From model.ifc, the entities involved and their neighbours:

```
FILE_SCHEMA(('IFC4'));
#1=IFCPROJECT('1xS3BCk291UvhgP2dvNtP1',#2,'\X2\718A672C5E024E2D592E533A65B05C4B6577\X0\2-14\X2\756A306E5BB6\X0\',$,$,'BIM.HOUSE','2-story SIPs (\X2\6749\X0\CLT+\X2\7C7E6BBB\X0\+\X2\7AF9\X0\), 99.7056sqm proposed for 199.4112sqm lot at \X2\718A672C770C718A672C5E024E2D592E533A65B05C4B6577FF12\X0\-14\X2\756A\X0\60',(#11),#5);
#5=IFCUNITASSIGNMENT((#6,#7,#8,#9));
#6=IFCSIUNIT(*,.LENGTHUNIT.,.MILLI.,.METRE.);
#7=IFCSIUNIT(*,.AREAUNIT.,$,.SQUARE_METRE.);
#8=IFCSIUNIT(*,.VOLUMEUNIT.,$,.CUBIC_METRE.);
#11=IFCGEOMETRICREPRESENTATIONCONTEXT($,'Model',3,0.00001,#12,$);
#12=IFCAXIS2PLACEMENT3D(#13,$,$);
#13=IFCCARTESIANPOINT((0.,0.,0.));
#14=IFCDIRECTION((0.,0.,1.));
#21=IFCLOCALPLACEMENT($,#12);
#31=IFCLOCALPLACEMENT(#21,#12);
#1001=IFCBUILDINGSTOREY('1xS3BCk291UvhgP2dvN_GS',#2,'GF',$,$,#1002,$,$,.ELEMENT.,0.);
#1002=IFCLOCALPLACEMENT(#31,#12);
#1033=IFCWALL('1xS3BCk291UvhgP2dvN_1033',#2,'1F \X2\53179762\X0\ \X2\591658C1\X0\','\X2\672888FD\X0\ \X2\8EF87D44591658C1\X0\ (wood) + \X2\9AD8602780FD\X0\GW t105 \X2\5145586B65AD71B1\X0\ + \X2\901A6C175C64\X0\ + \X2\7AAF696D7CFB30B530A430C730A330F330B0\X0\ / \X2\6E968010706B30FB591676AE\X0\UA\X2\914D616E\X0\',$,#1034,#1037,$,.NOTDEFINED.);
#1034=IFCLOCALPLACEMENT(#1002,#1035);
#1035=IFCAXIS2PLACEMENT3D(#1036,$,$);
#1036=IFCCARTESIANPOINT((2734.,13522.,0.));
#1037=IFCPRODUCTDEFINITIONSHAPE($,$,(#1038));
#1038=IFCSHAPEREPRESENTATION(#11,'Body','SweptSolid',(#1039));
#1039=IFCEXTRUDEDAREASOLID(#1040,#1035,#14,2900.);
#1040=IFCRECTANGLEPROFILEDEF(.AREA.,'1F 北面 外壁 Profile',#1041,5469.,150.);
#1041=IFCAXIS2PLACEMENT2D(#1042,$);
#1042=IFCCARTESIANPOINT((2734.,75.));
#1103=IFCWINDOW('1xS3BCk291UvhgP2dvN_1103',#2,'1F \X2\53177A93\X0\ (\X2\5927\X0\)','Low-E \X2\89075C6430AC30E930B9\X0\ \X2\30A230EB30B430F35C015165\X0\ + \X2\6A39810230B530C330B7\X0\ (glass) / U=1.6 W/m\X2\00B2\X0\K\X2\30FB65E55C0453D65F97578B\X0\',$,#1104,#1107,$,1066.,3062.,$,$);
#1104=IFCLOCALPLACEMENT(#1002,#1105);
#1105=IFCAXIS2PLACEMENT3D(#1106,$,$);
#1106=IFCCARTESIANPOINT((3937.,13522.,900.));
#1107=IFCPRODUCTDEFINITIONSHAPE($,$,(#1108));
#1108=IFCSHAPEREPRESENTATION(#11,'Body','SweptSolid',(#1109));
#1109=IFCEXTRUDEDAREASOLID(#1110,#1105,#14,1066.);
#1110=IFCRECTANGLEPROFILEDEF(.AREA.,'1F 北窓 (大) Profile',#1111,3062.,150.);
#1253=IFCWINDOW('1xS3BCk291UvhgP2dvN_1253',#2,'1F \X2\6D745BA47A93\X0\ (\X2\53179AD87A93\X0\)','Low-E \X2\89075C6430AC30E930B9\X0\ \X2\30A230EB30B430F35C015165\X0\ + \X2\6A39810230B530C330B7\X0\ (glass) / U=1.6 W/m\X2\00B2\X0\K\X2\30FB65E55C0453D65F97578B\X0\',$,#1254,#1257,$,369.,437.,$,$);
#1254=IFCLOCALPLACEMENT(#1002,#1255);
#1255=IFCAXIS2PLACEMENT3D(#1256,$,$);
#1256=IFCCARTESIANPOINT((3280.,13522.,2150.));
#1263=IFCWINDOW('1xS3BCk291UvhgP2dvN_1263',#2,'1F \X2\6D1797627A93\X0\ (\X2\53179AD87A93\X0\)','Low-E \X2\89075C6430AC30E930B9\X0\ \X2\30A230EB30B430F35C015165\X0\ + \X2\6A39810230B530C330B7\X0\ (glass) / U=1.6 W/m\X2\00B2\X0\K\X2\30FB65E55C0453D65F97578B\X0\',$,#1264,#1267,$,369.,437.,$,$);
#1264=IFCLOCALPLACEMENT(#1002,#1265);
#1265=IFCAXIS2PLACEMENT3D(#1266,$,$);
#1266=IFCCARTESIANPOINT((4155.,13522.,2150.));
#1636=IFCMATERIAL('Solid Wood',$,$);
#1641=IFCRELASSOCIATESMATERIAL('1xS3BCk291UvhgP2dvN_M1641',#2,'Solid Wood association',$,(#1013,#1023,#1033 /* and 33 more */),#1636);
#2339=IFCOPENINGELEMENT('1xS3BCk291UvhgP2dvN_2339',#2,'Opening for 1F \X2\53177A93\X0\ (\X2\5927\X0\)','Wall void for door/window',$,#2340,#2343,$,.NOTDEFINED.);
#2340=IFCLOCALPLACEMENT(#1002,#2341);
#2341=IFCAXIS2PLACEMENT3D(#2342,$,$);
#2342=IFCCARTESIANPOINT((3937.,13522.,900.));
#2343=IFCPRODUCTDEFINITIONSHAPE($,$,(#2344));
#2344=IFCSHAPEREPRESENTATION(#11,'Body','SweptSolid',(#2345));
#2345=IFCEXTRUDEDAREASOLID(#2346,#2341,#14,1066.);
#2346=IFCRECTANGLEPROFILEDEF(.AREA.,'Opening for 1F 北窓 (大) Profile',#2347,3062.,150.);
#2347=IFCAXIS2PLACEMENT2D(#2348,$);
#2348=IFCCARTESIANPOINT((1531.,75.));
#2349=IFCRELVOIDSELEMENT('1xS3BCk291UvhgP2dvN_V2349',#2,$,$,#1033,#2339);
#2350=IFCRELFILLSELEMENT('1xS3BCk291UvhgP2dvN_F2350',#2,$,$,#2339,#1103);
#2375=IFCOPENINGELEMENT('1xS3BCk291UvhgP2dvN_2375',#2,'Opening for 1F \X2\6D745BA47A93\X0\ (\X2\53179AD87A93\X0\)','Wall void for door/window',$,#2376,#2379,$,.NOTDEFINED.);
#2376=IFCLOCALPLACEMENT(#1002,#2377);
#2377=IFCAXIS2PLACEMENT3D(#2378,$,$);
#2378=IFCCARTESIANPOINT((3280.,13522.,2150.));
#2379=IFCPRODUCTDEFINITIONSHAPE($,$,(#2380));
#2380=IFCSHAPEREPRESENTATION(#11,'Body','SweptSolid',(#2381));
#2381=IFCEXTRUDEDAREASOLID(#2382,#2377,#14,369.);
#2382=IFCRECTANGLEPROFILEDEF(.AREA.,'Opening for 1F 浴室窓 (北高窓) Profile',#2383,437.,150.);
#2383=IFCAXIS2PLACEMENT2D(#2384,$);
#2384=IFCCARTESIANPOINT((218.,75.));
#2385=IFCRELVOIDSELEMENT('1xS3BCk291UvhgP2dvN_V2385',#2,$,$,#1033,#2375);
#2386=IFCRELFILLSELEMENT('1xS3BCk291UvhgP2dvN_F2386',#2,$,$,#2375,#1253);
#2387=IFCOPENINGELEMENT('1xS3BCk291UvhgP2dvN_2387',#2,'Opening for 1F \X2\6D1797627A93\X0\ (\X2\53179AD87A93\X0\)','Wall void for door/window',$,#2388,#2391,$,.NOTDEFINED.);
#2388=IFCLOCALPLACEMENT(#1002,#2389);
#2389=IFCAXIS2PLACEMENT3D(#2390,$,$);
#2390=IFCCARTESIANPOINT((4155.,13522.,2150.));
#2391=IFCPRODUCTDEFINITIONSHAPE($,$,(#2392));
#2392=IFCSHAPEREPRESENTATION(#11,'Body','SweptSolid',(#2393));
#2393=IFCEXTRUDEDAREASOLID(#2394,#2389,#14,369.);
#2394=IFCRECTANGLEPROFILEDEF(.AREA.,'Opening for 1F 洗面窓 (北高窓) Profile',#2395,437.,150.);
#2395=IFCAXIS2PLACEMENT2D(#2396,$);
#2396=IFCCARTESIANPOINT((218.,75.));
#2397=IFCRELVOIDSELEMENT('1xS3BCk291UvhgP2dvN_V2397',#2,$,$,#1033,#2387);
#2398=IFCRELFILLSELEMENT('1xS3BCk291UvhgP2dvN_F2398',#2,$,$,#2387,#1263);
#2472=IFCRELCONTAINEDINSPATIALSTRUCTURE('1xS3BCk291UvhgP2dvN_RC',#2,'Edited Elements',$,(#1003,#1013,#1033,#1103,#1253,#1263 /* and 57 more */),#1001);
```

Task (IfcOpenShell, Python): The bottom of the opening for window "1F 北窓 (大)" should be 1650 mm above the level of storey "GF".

```python
import numpy as np
import ifcopenshell
import ifcopenshell.api.geometry
import ifcopenshell.geom
import ifcopenshell.util.element
import ifcopenshell.util.placement
import ifcopenshell.util.shape
import ifcopenshell.util.unit

model = ifcopenshell.open("model.ifc")
unit_scale = ifcopenshell.util.unit.calculate_unit_scale(model)

window = model.by_id(1103)
opening = window.FillsVoids[0].RelatingOpeningElement
storey = ifcopenshell.util.element.get_container(window, ifc_class="IfcBuildingStorey")
level = ifcopenshell.util.placement.get_local_placement(storey.ObjectPlacement)[2, 3]

# The opening's origin need not be at the sill, so measure its lowest point.
shape = ifcopenshell.geom.create_shape(ifcopenshell.geom.settings(), opening)
bottom = ifcopenshell.util.shape.get_shape_bottom_elevation(shape, shape.geometry) / unit_scale
dz = level + 1.65 / unit_scale - bottom

shift = np.array([0.0, 0.0, dz])
# The window is not placed relative to its opening, so move both.
for product in (opening, window):
    matrix = ifcopenshell.util.placement.get_local_placement(product.ObjectPlacement)
    matrix[:3, 3] += shift
    ifcopenshell.api.geometry.edit_object_placement(model, product=product, matrix=matrix, is_si=False)

print(f"moved by {dz * unit_scale:+.3f} m")

model.write("model_updated.ifc")
```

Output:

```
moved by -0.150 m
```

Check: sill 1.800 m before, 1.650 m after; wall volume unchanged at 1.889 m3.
